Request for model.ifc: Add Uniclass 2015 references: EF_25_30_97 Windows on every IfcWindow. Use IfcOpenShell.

First a look at what the model holds.

```python
import ifcopenshell

model = ifcopenshell.open("model.ifc")
print(model.schema)
print("classifications:", [c.Name for c in model.by_type("IfcClassification")])
for ifc_class in ("IfcDoor", "IfcRoof", "IfcStair", "IfcWall", "IfcWindow"):
    print(ifc_class, len(model.by_type(ifc_class)))
```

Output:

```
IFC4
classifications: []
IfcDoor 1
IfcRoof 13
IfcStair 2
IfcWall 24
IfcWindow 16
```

```python
import ifcopenshell
import ifcopenshell.api.classification

model = ifcopenshell.open("model.ifc")

system = ifcopenshell.api.classification.add_classification(model, classification="Uniclass 2015")

codes = {
    "IfcWindow": ("EF_25_30_97", "Windows"),
}
for ifc_class, (code, name) in codes.items():
    products = model.by_type(ifc_class)
    ifcopenshell.api.classification.add_reference(
        model, products=products, classification=system, identification=code, name=name
    )
    print(code, len(products))

model.write("model_edited.ifc")
```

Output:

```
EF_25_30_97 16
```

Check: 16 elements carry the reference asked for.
